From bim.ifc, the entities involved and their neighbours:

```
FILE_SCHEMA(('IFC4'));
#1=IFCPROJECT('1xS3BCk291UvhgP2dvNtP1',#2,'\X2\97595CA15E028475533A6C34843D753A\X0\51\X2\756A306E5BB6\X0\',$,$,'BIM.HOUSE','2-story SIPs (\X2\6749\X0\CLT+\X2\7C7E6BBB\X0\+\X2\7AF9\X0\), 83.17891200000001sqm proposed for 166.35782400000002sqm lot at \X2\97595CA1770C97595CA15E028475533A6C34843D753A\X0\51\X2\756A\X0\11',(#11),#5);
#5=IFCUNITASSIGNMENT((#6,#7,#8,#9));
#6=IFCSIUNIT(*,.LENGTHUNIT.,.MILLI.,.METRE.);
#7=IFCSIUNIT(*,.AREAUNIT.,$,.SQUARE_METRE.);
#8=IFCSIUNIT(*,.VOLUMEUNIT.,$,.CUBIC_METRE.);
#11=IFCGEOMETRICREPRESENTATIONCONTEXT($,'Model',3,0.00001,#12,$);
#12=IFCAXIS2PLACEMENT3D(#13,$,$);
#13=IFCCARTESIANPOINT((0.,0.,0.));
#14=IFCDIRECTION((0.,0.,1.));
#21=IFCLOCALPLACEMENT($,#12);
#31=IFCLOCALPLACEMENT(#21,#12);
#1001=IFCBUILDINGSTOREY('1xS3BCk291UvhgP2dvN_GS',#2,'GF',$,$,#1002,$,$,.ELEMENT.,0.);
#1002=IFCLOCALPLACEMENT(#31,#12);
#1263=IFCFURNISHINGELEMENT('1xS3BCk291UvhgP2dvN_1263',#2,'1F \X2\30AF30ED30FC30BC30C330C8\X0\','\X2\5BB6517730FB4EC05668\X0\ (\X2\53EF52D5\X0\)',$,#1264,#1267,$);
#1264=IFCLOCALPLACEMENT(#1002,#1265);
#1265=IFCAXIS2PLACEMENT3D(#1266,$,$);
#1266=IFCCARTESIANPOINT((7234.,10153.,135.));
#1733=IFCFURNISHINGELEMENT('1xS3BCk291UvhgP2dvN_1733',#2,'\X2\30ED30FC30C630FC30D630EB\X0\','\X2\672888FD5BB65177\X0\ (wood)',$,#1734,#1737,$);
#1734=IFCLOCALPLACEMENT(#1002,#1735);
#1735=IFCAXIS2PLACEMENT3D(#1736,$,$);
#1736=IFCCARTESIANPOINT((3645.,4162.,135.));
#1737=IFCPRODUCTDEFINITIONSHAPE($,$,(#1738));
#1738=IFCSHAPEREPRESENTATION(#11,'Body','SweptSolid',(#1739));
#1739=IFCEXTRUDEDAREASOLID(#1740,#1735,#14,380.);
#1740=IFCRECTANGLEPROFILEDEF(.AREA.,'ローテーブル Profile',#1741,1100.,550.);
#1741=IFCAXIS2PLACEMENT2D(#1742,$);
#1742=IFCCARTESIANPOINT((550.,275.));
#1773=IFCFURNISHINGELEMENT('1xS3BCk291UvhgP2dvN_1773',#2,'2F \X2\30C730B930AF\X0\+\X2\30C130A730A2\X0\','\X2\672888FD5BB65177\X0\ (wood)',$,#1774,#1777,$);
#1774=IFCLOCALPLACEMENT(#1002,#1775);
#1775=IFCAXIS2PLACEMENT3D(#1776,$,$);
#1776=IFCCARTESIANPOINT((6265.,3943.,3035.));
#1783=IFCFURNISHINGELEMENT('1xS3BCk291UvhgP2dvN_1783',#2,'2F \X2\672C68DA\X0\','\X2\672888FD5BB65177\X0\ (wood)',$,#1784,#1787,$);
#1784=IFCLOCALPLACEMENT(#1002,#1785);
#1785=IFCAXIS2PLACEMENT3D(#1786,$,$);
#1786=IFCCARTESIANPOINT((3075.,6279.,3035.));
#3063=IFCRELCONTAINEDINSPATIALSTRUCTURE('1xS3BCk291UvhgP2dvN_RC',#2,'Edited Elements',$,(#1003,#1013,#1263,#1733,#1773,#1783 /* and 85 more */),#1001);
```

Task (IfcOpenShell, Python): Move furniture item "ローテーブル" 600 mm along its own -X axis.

```python
import ifcopenshell
import ifcopenshell.api.geometry
import ifcopenshell.util.placement
import ifcopenshell.util.unit

model = ifcopenshell.open("bim.ifc")
unit_scale = ifcopenshell.util.unit.calculate_unit_scale(model)

item = model.by_id(1733)
matrix = ifcopenshell.util.placement.get_local_placement(item.ObjectPlacement)
matrix[:3, 3] -= matrix[:3, 0] * 0.6 / unit_scale
ifcopenshell.api.geometry.edit_object_placement(model, product=item, matrix=matrix, is_si=False)

print(ifcopenshell.util.placement.get_local_placement(item.ObjectPlacement).round(3) + 0.0)

model.write("bim_edited.ifc")
```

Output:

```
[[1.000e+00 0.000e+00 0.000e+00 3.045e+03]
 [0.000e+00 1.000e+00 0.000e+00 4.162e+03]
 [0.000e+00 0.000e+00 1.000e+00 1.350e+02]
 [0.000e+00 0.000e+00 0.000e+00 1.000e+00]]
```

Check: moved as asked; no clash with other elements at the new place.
